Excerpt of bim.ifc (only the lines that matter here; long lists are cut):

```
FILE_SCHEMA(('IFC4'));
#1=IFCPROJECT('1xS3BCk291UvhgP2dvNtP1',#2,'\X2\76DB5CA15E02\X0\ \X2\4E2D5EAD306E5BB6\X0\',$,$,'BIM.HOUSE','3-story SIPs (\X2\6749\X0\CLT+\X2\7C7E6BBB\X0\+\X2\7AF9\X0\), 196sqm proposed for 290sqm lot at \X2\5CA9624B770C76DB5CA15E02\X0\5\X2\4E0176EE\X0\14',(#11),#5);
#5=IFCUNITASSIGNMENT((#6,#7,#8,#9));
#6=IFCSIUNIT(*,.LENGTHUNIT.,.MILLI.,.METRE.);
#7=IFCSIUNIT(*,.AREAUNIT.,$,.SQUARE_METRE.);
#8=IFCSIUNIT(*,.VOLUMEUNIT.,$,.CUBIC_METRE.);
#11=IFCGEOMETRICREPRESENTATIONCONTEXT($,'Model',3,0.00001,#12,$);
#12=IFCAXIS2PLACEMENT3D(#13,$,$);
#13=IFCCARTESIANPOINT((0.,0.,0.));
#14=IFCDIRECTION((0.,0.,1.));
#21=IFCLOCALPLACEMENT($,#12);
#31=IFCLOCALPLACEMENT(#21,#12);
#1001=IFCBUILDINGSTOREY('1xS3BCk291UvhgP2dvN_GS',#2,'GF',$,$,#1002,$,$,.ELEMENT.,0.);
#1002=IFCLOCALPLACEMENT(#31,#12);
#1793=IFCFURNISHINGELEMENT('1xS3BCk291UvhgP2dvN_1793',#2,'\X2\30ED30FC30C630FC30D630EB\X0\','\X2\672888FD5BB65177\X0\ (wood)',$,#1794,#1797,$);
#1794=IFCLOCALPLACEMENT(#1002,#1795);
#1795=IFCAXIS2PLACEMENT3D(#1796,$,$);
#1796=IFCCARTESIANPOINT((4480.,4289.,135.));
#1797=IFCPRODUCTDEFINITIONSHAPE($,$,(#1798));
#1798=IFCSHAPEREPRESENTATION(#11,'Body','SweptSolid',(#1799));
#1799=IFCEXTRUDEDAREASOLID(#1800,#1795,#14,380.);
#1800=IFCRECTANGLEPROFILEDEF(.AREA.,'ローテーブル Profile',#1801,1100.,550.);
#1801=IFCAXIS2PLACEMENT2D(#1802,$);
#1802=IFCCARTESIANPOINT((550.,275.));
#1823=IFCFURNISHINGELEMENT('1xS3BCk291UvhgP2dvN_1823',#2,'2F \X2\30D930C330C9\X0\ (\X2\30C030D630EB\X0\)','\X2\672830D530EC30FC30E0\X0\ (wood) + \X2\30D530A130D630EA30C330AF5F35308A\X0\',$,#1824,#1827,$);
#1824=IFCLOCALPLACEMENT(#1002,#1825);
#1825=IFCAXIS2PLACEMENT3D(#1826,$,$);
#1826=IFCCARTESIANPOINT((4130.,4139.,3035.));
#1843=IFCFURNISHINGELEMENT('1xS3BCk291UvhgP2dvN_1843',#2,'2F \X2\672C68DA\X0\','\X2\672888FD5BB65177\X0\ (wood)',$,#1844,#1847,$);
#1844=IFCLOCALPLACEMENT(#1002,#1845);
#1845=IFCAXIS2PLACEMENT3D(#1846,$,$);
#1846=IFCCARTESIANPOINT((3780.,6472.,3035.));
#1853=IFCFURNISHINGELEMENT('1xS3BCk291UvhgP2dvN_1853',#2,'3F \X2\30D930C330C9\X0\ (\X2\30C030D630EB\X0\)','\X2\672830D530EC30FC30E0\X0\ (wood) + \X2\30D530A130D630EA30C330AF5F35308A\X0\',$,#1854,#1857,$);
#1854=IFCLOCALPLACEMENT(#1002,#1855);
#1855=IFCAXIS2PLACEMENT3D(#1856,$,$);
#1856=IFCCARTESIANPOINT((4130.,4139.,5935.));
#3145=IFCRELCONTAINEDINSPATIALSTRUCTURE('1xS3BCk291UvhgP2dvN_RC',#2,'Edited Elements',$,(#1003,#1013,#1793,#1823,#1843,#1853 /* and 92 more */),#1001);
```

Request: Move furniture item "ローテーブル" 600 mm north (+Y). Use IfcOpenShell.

```python
import ifcopenshell
import ifcopenshell.api.geometry
import ifcopenshell.util.placement
import ifcopenshell.util.unit

model = ifcopenshell.open("bim.ifc")
unit_scale = ifcopenshell.util.unit.calculate_unit_scale(model)

item = model.by_guid("1xS3BCk291UvhgP2dvN_1793")
matrix = ifcopenshell.util.placement.get_local_placement(item.ObjectPlacement)
matrix[1, 3] += 0.6 / unit_scale
ifcopenshell.api.geometry.edit_object_placement(model, product=item, matrix=matrix, is_si=False)

print(ifcopenshell.util.placement.get_local_placement(item.ObjectPlacement).round(3) + 0.0)

model.write("bim_rev.ifc")
```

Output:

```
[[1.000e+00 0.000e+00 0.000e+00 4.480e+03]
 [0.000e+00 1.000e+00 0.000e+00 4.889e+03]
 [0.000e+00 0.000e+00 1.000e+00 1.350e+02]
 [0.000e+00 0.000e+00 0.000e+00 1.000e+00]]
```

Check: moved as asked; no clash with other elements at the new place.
